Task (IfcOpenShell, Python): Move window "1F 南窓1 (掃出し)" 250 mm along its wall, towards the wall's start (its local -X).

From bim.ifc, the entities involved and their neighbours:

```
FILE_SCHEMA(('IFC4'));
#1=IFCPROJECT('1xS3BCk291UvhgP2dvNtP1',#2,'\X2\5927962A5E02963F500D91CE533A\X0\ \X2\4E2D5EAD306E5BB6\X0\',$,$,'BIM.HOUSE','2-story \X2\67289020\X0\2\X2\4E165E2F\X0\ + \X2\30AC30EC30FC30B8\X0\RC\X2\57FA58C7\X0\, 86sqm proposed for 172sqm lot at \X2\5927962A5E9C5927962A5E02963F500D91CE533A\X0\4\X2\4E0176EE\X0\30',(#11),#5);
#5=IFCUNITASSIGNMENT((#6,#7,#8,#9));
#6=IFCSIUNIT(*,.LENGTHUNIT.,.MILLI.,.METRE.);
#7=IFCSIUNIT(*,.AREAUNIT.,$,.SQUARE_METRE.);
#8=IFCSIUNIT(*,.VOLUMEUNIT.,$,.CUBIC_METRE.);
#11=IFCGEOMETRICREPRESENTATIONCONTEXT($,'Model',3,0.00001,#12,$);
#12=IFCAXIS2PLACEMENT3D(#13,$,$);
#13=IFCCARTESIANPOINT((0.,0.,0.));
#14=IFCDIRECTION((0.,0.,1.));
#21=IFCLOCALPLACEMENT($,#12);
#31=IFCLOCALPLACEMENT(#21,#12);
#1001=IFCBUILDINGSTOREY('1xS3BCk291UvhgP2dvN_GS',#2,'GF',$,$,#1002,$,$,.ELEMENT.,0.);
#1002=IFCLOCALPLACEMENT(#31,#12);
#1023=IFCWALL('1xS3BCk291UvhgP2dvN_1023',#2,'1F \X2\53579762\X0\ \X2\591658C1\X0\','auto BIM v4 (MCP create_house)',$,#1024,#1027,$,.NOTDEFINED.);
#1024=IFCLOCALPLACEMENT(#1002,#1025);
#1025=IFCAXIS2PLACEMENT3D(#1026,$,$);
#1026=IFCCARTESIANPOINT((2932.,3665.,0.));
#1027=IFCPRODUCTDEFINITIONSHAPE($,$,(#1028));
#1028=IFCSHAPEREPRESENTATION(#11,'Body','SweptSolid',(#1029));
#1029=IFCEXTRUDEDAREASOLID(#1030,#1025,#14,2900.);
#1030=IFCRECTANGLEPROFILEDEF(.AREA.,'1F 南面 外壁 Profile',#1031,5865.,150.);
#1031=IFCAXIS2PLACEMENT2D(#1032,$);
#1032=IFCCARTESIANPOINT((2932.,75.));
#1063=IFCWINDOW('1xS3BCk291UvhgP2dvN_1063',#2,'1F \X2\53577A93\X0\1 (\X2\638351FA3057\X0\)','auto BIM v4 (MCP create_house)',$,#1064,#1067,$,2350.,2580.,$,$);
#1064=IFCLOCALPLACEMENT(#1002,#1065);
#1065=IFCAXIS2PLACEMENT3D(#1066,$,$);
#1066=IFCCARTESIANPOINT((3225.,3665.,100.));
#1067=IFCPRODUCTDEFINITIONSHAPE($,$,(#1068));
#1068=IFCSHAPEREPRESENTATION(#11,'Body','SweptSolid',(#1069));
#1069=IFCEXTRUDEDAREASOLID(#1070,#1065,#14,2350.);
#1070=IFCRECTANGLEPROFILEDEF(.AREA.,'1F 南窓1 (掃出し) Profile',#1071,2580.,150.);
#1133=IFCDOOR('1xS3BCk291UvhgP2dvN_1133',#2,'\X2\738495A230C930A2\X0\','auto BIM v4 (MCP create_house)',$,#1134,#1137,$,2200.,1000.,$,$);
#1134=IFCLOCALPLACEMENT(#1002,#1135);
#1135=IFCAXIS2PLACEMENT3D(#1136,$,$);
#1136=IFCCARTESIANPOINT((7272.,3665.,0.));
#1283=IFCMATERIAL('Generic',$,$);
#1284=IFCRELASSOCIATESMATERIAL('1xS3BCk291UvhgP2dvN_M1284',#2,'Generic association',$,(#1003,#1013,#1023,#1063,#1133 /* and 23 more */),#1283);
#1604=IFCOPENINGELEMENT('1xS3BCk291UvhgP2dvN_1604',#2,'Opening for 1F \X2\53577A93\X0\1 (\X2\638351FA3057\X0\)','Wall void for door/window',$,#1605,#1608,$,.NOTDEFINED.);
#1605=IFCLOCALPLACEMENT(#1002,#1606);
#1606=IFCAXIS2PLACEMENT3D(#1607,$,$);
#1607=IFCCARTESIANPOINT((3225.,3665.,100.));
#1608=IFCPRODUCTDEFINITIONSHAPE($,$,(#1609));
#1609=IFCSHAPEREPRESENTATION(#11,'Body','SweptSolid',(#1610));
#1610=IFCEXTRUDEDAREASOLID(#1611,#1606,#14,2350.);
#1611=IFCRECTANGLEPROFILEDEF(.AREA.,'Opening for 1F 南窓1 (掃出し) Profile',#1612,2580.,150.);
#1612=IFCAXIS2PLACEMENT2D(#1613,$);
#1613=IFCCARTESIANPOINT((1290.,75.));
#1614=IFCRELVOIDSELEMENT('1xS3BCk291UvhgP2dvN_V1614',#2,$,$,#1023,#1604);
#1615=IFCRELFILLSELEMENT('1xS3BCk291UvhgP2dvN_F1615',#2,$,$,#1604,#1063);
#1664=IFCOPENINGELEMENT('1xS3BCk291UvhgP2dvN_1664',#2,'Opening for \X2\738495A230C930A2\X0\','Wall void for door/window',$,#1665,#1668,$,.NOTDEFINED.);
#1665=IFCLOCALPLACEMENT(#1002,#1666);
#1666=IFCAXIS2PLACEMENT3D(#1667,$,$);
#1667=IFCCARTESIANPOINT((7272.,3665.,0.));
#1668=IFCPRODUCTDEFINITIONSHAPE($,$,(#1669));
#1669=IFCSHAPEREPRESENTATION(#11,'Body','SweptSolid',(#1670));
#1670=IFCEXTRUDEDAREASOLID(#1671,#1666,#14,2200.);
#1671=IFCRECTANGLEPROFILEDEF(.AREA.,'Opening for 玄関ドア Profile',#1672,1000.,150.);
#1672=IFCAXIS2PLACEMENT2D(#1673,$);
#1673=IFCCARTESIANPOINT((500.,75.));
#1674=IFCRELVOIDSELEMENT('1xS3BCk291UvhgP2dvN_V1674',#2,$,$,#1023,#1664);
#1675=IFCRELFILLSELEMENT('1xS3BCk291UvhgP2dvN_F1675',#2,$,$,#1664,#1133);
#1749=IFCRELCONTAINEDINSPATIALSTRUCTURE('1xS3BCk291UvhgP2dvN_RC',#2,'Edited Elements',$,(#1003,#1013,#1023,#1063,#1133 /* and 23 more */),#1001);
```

```python
import ifcopenshell
import ifcopenshell.api.geometry
import ifcopenshell.util.placement
import ifcopenshell.util.unit

model = ifcopenshell.open("bim.ifc")
unit_scale = ifcopenshell.util.unit.calculate_unit_scale(model)

window = model.by_guid("1xS3BCk291UvhgP2dvN_1063")
opening = window.FillsVoids[0].RelatingOpeningElement
wall = opening.VoidsElements[0].RelatingBuildingElement

wall_matrix = ifcopenshell.util.placement.get_local_placement(wall.ObjectPlacement)
shift = wall_matrix[:3, 0] * -0.25 / unit_scale
before = ifcopenshell.util.placement.get_local_placement(window.ObjectPlacement)[:3, 3].copy()

# The window is not placed relative to its opening, so move both.
for product in (opening, window):
    matrix = ifcopenshell.util.placement.get_local_placement(product.ObjectPlacement)
    matrix[:3, 3] += shift
    ifcopenshell.api.geometry.edit_object_placement(model, product=product, matrix=matrix, is_si=False)

after = ifcopenshell.util.placement.get_local_placement(window.ObjectPlacement)[:3, 3]
print("window moved by", (after - before).round(3) + 0.0)

model.write("bim_updated.ifc")
```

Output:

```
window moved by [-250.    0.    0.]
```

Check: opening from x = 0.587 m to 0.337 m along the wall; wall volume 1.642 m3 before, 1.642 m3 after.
